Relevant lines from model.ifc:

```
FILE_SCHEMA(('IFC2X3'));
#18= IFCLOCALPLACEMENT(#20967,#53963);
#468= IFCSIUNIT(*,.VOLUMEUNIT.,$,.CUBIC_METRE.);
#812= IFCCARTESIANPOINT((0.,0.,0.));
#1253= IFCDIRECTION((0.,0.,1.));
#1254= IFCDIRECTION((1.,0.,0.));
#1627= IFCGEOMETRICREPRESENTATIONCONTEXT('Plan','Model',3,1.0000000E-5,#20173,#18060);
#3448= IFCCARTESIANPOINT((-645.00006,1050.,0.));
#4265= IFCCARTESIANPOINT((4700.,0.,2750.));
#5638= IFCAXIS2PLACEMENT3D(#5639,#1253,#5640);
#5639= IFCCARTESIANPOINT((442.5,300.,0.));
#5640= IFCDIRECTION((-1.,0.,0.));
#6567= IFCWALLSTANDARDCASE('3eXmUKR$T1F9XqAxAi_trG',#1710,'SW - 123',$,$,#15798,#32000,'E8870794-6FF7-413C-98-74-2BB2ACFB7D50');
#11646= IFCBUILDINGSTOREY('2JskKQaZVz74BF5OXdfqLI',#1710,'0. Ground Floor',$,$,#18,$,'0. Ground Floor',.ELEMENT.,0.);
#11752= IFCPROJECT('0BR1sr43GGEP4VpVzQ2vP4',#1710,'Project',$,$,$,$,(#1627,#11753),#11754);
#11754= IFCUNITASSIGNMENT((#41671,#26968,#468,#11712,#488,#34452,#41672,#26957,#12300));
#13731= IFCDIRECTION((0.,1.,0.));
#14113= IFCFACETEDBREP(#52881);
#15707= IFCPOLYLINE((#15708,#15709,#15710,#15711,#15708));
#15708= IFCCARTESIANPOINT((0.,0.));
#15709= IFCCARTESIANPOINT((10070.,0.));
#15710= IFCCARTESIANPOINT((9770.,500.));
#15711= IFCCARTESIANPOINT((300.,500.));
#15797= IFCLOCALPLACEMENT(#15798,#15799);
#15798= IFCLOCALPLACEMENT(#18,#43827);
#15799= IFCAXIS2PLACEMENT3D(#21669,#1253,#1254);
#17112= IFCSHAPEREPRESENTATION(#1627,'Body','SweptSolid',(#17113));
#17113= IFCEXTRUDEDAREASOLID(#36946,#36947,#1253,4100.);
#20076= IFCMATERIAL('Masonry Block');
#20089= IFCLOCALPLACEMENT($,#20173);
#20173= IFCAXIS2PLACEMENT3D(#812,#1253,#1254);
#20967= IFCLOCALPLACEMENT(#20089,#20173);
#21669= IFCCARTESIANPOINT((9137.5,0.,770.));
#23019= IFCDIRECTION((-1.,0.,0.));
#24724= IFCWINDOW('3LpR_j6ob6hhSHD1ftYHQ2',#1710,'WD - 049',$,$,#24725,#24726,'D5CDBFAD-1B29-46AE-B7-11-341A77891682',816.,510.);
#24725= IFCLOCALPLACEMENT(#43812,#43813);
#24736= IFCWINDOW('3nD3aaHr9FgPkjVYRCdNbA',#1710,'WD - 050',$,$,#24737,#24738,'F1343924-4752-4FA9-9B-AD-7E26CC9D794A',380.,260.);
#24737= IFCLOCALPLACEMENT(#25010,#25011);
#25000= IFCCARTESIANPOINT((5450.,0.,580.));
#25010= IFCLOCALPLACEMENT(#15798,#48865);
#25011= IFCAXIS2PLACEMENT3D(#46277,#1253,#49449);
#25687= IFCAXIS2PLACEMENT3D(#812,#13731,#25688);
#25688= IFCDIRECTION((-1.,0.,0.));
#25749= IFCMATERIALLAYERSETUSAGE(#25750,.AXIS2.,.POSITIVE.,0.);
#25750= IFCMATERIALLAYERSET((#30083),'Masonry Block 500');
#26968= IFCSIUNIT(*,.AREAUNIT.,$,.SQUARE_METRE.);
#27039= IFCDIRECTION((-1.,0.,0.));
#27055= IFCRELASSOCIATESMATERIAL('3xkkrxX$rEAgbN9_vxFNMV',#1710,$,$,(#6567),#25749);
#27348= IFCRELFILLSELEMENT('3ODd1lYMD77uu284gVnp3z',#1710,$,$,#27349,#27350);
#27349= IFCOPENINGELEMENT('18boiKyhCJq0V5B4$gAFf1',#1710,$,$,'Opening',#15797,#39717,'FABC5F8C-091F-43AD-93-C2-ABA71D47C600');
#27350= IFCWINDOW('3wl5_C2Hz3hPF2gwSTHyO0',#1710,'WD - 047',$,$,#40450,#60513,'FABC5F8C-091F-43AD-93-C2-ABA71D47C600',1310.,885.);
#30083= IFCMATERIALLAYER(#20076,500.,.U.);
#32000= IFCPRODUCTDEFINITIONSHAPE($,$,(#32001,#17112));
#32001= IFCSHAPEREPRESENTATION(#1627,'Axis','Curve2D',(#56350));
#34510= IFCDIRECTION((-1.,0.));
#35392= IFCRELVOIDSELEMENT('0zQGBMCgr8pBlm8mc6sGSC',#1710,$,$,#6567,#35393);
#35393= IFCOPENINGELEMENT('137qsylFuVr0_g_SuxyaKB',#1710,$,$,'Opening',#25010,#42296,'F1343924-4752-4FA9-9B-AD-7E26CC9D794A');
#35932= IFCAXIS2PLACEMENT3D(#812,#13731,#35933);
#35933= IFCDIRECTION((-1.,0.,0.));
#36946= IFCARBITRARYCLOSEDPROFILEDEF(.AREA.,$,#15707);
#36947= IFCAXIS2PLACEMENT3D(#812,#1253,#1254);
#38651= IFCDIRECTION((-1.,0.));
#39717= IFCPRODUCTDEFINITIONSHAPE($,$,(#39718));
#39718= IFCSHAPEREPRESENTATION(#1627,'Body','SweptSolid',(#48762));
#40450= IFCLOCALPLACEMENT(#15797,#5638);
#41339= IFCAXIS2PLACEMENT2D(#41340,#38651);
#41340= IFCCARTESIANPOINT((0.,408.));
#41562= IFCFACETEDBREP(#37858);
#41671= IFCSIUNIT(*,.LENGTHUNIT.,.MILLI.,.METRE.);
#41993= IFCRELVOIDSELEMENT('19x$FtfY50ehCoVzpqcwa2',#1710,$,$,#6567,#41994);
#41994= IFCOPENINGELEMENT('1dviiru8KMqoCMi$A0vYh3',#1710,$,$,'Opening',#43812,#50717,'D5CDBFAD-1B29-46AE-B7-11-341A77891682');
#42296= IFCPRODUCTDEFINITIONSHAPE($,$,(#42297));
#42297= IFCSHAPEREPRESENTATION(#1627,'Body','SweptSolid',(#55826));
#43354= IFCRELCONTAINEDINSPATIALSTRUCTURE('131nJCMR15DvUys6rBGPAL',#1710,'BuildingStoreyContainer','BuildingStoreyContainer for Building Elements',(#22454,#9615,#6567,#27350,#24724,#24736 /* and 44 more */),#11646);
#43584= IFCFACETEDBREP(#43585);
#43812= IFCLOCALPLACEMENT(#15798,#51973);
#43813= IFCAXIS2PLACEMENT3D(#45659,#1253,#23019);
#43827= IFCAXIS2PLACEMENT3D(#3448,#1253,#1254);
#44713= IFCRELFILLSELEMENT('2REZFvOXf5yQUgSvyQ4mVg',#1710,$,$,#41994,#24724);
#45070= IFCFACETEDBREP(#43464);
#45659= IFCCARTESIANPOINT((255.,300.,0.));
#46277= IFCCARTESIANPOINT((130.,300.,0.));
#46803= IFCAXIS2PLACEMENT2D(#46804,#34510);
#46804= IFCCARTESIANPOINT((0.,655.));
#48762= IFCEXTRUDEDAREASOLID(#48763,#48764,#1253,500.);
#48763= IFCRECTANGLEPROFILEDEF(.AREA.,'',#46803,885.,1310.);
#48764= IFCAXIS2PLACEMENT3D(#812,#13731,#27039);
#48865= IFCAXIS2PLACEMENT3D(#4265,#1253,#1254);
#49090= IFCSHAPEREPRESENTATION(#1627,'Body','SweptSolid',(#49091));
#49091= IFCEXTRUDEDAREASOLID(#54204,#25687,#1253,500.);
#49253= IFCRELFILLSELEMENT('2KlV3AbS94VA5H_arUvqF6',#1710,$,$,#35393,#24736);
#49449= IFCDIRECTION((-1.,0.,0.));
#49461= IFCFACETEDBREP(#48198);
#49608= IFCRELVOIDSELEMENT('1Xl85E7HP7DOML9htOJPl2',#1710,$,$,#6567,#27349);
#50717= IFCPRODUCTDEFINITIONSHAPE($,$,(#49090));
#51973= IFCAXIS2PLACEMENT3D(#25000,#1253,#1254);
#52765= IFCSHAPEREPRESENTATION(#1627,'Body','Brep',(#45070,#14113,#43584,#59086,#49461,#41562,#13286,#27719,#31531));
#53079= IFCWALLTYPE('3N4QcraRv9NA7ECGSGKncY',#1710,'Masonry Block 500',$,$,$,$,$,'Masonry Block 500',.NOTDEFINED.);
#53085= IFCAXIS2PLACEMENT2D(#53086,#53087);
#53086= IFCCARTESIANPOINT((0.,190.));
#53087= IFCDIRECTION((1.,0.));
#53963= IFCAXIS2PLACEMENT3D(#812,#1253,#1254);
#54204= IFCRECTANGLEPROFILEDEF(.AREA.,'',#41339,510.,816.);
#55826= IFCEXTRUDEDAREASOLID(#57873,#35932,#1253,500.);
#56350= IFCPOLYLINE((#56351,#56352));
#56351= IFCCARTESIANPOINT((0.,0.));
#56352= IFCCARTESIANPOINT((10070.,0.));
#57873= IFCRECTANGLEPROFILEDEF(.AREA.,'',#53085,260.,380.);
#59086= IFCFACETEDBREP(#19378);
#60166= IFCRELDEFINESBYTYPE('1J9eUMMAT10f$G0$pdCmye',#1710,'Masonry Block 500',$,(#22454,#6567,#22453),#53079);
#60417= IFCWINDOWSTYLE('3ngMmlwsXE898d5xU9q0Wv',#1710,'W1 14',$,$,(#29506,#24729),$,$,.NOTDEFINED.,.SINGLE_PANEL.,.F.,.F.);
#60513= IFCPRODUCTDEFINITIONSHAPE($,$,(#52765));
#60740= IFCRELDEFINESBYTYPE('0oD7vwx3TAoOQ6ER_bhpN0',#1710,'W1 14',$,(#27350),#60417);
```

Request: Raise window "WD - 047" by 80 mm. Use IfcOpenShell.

```python
import numpy as np
import ifcopenshell
import ifcopenshell.api.geometry
import ifcopenshell.util.placement
import ifcopenshell.util.unit

model = ifcopenshell.open("model.ifc")
unit_scale = ifcopenshell.util.unit.calculate_unit_scale(model)

window = model.by_guid("3wl5_C2Hz3hPF2gwSTHyO0")
opening = window.FillsVoids[0].RelatingOpeningElement
dz = 0.08 / unit_scale

shift = np.array([0.0, 0.0, dz])
# The window is placed relative to its opening, so it follows when the opening moves.
matrix = ifcopenshell.util.placement.get_local_placement(opening.ObjectPlacement)
matrix[:3, 3] += shift
ifcopenshell.api.geometry.edit_object_placement(
    model, product=opening, matrix=matrix, is_si=False, should_transform_children=True
)

print(f"moved by {dz * unit_scale:+.3f} m")

model.write("model_v2.ifc")
```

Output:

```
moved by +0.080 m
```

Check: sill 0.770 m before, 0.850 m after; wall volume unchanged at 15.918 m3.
